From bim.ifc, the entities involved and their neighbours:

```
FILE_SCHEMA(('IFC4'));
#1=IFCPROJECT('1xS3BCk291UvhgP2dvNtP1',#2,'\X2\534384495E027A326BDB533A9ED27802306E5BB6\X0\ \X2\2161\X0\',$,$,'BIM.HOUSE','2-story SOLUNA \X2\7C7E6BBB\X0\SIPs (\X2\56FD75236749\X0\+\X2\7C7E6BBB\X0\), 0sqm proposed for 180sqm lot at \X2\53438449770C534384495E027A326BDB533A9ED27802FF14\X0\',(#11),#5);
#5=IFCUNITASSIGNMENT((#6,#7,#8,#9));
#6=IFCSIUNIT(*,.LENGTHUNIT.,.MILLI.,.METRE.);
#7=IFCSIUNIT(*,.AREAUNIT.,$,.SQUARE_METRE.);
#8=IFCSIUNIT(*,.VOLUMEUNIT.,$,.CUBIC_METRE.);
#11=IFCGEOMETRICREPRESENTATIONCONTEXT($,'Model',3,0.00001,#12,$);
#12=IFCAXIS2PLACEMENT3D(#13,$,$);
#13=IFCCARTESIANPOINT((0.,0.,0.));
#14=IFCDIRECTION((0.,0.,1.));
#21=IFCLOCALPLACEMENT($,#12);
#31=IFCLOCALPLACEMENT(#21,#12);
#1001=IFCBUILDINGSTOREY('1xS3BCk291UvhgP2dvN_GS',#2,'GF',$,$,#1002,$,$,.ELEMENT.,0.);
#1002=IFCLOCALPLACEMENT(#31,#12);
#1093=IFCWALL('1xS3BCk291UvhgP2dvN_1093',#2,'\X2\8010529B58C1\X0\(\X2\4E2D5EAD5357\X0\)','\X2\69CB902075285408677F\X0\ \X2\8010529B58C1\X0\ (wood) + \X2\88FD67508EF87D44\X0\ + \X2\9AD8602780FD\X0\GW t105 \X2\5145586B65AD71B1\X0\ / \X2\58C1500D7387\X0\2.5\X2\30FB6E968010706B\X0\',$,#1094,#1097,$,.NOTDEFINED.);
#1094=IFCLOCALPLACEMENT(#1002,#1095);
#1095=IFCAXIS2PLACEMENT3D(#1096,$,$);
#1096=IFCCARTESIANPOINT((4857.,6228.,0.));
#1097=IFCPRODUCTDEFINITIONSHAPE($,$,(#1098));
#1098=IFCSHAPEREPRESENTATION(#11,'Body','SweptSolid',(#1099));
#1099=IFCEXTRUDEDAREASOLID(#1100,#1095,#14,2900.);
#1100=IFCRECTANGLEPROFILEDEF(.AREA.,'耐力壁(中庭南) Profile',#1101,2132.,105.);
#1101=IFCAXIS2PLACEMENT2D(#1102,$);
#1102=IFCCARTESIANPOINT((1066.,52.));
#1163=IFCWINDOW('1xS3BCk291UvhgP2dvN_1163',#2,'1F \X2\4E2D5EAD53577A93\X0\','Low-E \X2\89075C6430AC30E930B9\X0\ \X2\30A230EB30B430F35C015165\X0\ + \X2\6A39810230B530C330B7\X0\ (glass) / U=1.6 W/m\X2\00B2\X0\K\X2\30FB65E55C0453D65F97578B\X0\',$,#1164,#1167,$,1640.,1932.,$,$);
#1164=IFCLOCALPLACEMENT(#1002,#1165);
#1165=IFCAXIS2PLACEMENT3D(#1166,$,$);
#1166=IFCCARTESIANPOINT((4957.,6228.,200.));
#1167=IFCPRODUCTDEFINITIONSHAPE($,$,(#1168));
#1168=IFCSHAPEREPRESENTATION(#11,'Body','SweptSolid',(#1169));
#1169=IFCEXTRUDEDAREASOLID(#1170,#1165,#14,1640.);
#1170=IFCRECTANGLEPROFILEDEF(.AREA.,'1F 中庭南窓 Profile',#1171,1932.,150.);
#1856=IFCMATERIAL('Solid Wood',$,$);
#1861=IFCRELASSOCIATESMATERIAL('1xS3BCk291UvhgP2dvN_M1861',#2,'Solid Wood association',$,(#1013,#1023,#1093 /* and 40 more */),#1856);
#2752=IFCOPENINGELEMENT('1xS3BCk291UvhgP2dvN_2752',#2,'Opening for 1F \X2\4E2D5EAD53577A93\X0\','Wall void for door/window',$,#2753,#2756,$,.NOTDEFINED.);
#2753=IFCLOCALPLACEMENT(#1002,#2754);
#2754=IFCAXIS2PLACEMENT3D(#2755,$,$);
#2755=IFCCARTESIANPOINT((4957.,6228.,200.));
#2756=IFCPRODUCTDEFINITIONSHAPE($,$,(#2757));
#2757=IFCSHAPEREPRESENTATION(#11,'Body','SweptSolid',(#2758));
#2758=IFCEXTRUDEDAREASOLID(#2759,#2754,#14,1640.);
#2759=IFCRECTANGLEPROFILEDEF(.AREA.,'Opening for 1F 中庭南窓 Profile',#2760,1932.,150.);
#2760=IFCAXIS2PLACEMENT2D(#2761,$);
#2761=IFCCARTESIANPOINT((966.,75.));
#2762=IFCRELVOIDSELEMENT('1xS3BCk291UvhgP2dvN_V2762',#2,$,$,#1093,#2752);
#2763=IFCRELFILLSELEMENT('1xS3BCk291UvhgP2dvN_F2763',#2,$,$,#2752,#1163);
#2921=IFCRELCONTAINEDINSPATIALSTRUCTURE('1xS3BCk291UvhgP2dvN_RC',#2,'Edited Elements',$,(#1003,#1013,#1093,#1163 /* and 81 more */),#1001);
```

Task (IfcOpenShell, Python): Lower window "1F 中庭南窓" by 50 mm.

```python
import numpy as np
import ifcopenshell
import ifcopenshell.api.geometry
import ifcopenshell.util.placement
import ifcopenshell.util.unit

model = ifcopenshell.open("bim.ifc")
unit_scale = ifcopenshell.util.unit.calculate_unit_scale(model)

window = model.by_guid("1xS3BCk291UvhgP2dvN_1163")
opening = window.FillsVoids[0].RelatingOpeningElement
dz = -50.0

shift = np.array([0.0, 0.0, dz])
# The window is not placed relative to its opening, so move both.
for product in (opening, window):
    matrix = ifcopenshell.util.placement.get_local_placement(product.ObjectPlacement)
    matrix[:3, 3] += shift
    ifcopenshell.api.geometry.edit_object_placement(model, product=product, matrix=matrix, is_si=False)

print(f"moved by {dz * unit_scale:+.3f} m")

model.write("bim_rev.ifc")
```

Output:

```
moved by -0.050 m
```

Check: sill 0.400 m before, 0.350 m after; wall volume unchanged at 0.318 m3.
